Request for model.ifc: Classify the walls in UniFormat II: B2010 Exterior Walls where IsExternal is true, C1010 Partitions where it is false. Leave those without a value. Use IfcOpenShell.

First a look at what the model holds.

```python
import ifcopenshell
import ifcopenshell.util.element

model = ifcopenshell.open("model.ifc")
print(model.schema)
print("classifications:", [c.Name for c in model.by_type("IfcClassification")])
values = [ifcopenshell.util.element.get_pset(e, "Pset_WallCommon", "IsExternal") for e in model.by_type("IfcWall")]
for value in (True, False, None):
    print("IsExternal", value, values.count(value))
```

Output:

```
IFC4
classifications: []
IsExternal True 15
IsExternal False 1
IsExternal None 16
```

```python
import ifcopenshell
import ifcopenshell.api.classification
import ifcopenshell.util.element

model = ifcopenshell.open("model.ifc")

system = ifcopenshell.api.classification.add_classification(model, classification="UniFormat II")

walls = model.by_type("IfcWall")
external = {e: ifcopenshell.util.element.get_pset(e, "Pset_WallCommon", "IsExternal") for e in walls}
for flag, code, name in ((True, "B2010", "Exterior Walls"), (False, "C1010", "Partitions")):
    products = [e for e in walls if external[e] is flag]
    ifcopenshell.api.classification.add_reference(
        model, products=products, classification=system, identification=code, name=name
    )
    print(code, len(products))

model.write("model_updated.ifc")
```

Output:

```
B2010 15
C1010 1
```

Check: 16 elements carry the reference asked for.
